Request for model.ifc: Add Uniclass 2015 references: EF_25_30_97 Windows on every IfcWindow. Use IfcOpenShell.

First a look at what the model holds.

```python
import ifcopenshell

model = ifcopenshell.open("model.ifc")
print(model.schema)
print("classifications:", [c.Name for c in model.by_type("IfcClassification")])
for ifc_class in ("IfcDoor", "IfcRoof", "IfcStair", "IfcWall", "IfcWindow"):
    print(ifc_class, len(model.by_type(ifc_class)))
```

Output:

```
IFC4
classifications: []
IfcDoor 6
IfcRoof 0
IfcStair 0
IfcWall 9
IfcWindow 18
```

```python
import ifcopenshell
import ifcopenshell.api.classification

model = ifcopenshell.open("model.ifc")

system = ifcopenshell.api.classification.add_classification(model, classification="Uniclass 2015")

codes = {
    "IfcWindow": ("EF_25_30_97", "Windows"),
}
for ifc_class, (code, name) in codes.items():
    products = model.by_type(ifc_class)
    ifcopenshell.api.classification.add_reference(
        model, products=products, classification=system, identification=code, name=name
    )
    print(code, len(products))

model.write("model_v2.ifc")
```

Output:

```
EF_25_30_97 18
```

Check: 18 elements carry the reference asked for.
